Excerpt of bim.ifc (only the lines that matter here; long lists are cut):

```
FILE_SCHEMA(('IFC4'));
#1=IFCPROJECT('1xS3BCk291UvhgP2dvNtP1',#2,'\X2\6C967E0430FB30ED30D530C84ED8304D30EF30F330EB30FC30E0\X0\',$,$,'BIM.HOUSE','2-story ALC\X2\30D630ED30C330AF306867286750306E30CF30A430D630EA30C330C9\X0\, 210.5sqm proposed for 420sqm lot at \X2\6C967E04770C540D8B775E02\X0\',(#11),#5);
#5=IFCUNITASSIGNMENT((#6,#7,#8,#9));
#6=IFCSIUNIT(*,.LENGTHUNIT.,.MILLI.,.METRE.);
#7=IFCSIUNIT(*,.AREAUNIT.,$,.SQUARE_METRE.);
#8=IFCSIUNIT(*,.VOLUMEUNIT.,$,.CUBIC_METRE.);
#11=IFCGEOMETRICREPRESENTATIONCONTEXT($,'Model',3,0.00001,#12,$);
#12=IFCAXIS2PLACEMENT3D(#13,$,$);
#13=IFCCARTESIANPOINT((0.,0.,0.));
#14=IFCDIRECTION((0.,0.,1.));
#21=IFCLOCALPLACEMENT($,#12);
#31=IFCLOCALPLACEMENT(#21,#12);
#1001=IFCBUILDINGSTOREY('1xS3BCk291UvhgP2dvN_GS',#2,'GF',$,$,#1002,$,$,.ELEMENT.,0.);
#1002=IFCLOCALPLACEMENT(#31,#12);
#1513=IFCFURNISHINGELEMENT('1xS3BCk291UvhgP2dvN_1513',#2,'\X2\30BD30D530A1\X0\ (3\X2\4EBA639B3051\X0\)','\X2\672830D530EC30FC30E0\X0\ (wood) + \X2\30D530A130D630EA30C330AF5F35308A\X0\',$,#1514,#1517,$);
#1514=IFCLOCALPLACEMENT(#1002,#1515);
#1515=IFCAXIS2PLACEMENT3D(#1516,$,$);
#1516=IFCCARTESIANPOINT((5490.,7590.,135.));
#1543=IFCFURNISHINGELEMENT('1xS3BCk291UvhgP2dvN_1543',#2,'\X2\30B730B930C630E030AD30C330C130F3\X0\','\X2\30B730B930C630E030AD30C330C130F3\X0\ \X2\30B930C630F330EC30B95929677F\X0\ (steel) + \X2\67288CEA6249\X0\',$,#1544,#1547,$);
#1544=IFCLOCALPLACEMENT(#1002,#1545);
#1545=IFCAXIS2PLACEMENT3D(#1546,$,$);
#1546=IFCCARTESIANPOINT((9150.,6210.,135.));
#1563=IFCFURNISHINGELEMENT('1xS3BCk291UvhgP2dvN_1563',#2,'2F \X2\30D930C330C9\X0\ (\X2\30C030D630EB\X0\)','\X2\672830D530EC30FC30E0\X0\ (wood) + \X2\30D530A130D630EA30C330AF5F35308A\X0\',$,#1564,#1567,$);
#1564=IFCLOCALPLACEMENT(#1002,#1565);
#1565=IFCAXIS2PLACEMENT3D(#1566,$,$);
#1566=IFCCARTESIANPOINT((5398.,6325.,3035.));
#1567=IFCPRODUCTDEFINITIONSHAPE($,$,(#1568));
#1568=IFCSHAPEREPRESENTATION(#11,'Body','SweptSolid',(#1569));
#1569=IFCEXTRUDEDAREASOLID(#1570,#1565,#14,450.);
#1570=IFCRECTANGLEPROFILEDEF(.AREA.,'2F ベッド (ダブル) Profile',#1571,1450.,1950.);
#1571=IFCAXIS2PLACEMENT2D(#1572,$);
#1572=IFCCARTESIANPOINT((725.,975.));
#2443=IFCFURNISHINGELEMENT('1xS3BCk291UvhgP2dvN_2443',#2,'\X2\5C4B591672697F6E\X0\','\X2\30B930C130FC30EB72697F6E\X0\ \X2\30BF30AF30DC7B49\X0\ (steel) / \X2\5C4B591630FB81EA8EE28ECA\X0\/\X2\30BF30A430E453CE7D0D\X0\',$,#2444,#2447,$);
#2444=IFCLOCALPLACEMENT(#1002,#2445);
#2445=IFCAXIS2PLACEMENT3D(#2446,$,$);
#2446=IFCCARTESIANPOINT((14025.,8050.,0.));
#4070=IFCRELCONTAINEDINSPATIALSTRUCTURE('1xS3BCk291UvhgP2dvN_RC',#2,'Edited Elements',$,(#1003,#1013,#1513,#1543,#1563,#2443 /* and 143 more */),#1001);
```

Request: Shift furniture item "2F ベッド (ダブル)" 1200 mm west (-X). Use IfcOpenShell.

```python
import ifcopenshell
import ifcopenshell.api.geometry
import ifcopenshell.util.placement
import ifcopenshell.util.unit

model = ifcopenshell.open("bim.ifc")
unit_scale = ifcopenshell.util.unit.calculate_unit_scale(model)

item = model.by_guid("1xS3BCk291UvhgP2dvN_1563")
matrix = ifcopenshell.util.placement.get_local_placement(item.ObjectPlacement)
matrix[0, 3] -= 1.2 / unit_scale
ifcopenshell.api.geometry.edit_object_placement(model, product=item, matrix=matrix, is_si=False)

print(ifcopenshell.util.placement.get_local_placement(item.ObjectPlacement).round(3) + 0.0)

model.write("bim_updated.ifc")
```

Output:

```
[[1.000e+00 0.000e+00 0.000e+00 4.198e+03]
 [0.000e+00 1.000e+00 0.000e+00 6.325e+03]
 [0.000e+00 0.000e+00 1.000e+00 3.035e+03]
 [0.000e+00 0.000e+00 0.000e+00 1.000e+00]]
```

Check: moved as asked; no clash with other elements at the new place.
